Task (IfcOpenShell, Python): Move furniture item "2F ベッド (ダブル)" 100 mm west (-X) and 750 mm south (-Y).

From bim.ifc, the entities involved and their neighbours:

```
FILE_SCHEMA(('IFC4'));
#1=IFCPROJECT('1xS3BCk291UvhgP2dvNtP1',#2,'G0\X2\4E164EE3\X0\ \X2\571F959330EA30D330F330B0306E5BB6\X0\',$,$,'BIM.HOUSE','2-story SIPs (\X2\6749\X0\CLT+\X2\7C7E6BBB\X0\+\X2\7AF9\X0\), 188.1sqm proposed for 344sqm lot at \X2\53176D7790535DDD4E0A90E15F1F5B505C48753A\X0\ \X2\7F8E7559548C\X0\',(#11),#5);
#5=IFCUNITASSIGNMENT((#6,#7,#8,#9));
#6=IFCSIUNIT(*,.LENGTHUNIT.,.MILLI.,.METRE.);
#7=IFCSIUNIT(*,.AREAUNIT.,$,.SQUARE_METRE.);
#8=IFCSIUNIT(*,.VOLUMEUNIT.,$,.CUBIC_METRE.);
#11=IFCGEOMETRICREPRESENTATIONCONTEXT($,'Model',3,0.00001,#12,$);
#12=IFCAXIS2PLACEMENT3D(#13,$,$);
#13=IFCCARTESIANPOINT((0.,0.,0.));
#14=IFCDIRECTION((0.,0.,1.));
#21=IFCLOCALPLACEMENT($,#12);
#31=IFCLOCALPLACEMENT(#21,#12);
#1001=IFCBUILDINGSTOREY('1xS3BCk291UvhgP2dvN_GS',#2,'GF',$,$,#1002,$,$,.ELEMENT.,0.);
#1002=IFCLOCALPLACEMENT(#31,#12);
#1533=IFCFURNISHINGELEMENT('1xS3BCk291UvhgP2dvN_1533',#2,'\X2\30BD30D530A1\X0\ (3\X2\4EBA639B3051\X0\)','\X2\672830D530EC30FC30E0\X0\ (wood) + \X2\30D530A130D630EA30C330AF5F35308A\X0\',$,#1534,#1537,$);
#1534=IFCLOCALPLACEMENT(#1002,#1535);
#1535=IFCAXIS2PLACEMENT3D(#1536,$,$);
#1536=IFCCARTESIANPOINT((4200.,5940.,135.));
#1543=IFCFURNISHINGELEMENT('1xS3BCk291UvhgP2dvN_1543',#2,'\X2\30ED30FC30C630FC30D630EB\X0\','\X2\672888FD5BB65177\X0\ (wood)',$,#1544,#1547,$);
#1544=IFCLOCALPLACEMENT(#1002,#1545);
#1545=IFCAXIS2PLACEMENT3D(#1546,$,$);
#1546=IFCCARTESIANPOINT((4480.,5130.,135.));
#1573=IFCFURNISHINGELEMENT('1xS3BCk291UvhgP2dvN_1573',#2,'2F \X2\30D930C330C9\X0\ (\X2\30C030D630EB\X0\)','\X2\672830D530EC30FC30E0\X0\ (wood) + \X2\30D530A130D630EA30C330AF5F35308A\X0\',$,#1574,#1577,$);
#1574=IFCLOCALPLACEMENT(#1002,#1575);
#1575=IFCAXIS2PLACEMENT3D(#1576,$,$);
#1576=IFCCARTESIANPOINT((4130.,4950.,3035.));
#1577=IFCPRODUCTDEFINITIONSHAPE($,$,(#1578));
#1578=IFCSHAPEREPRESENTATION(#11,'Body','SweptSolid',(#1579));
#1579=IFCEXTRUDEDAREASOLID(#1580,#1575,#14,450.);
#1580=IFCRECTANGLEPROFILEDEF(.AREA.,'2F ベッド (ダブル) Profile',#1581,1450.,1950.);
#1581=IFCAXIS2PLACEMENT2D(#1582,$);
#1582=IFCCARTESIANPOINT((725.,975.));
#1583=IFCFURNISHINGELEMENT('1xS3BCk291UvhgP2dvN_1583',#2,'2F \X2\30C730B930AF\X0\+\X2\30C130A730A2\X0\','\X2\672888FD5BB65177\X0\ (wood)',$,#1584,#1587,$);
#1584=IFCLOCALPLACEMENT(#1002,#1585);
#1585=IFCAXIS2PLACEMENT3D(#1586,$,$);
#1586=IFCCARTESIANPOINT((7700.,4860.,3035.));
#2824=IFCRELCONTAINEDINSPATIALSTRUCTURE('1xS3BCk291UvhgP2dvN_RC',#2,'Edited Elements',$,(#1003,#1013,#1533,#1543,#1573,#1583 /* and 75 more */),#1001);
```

```python
import ifcopenshell
import ifcopenshell.api.geometry
import ifcopenshell.util.placement
import ifcopenshell.util.unit

model = ifcopenshell.open("bim.ifc")
unit_scale = ifcopenshell.util.unit.calculate_unit_scale(model)

item = model.by_id(1573)
matrix = ifcopenshell.util.placement.get_local_placement(item.ObjectPlacement)
matrix[0, 3] -= 0.1 / unit_scale
matrix[1, 3] -= 0.75 / unit_scale
ifcopenshell.api.geometry.edit_object_placement(model, product=item, matrix=matrix, is_si=False)

print(ifcopenshell.util.placement.get_local_placement(item.ObjectPlacement).round(3) + 0.0)

model.write("bim-out.ifc")
```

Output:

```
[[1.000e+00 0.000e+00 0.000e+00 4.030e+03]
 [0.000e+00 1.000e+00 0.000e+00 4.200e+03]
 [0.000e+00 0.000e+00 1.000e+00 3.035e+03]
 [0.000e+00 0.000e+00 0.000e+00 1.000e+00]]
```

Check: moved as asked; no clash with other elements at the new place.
